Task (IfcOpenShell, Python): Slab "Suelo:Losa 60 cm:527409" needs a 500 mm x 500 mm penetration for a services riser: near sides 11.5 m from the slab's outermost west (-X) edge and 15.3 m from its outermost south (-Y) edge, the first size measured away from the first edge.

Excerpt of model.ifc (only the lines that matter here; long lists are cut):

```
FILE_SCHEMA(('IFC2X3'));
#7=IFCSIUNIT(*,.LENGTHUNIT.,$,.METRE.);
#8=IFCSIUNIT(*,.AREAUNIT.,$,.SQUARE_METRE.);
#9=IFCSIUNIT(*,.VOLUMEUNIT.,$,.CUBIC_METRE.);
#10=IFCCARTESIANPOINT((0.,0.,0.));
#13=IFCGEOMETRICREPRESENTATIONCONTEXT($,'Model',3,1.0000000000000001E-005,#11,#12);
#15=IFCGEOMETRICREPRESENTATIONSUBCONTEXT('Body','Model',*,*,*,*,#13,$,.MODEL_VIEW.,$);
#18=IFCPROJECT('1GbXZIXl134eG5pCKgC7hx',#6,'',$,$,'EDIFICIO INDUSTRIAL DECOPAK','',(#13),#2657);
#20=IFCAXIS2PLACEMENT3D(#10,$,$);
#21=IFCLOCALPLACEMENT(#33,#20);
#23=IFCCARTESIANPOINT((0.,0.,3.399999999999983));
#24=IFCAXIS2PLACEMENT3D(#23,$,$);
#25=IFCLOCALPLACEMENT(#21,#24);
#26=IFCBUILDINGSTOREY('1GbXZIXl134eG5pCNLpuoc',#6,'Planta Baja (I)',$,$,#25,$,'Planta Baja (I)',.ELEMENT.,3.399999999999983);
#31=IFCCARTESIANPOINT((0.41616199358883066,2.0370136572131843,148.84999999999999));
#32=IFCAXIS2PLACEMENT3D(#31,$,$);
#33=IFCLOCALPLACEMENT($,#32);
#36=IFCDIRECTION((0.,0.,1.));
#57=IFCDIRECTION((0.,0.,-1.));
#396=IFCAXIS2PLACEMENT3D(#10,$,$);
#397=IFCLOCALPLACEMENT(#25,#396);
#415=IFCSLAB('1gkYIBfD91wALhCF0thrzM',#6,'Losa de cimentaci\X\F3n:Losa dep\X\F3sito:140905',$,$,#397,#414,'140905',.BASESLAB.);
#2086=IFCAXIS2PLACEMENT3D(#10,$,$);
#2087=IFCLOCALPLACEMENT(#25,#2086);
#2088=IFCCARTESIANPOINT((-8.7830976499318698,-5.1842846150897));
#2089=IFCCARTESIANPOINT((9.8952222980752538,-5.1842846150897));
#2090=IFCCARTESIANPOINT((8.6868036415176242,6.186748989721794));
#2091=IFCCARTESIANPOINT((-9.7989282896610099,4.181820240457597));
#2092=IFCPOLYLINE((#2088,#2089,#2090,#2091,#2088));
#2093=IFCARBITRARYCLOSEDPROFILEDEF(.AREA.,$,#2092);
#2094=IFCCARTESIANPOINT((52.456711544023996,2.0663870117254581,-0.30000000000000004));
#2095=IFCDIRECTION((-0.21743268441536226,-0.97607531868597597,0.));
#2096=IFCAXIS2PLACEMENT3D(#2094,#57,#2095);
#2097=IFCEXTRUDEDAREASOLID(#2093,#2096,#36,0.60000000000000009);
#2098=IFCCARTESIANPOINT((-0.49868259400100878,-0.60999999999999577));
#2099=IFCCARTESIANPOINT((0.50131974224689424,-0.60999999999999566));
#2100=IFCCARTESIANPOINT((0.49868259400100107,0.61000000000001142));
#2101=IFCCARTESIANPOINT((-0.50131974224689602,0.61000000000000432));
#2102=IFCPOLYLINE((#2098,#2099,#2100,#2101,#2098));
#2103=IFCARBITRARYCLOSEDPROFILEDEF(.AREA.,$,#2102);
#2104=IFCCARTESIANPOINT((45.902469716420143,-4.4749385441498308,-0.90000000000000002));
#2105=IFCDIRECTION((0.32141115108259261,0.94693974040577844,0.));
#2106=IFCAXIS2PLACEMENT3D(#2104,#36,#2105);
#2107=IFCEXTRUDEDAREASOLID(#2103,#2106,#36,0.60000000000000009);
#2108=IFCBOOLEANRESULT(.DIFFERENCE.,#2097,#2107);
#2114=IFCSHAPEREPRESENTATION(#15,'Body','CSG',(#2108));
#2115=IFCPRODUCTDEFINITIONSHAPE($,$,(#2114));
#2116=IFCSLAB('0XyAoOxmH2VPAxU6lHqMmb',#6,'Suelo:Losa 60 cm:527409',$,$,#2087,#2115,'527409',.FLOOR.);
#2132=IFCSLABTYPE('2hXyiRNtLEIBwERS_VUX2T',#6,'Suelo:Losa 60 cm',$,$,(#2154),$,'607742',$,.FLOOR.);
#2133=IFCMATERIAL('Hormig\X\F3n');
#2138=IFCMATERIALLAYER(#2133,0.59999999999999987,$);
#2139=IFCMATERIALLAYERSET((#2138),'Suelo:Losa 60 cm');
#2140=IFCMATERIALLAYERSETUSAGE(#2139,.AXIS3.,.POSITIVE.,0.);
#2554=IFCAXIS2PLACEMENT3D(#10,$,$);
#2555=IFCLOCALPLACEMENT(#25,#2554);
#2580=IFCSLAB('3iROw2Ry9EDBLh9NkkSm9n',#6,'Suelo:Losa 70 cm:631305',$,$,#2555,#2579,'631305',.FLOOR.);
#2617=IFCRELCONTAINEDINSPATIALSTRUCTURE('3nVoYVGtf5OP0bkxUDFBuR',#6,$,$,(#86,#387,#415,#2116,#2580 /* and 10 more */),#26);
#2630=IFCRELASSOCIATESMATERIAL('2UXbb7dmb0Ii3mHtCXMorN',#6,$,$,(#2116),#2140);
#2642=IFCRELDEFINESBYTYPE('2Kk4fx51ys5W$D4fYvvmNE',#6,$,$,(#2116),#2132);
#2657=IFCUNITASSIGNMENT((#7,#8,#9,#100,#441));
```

```python
import numpy as np
import ifcopenshell
import ifcopenshell.api.feature
import ifcopenshell.api.geometry
import ifcopenshell.api.root
import ifcopenshell.geom
import ifcopenshell.util.placement
import ifcopenshell.util.representation
import ifcopenshell.util.shape
import ifcopenshell.util.unit

model = ifcopenshell.open("model.ifc")
unit_scale = ifcopenshell.util.unit.calculate_unit_scale(model)
settings = ifcopenshell.geom.settings()


def volume(element):
    """Net volume in cubic metres, openings subtracted."""
    shape = ifcopenshell.geom.create_shape(settings, element)
    return ifcopenshell.util.shape.get_volume(shape.geometry)


slab = model.by_id(2116)
before = volume(slab)

# Extent in the slab's own axes, in metres. The edges named are its -X and -Y sides.
slab_shape = ifcopenshell.geom.create_shape(settings, slab)
vertices = ifcopenshell.util.shape.get_vertices(slab_shape.geometry)
x_min, y_min, bottom = vertices.min(axis=0)
top = vertices[:, 2].max()

opening = ifcopenshell.api.root.create_entity(model, ifc_class="IfcOpeningElement", name="Services riser opening")
context = ifcopenshell.util.representation.get_context(model, "Model", "Body", "MODEL_VIEW")
width, depth = 0.5, 0.5
outline = [(0.0, 0.0), (width, 0.0), (width, depth), (0.0, depth), (0.0, 0.0)]
# Overshoot both faces by 50 mm so the cut is clean.
shape = ifcopenshell.api.geometry.add_slab_representation(
    model, context=context, depth=top - bottom + 0.1, polyline=outline
)
ifcopenshell.api.geometry.assign_representation(model, product=opening, representation=shape)

matrix = ifcopenshell.util.placement.get_local_placement(slab.ObjectPlacement)
matrix[:, 3] = matrix @ np.append(np.array([x_min + 11.5, y_min + 15.3, bottom - 0.05]) / unit_scale, 1.0)
ifcopenshell.api.geometry.edit_object_placement(model, product=opening, matrix=matrix, is_si=False)
ifcopenshell.api.feature.add_feature(model, feature=opening, element=slab)

after = volume(slab)

print(f"slab volume {before:.3f} -> {after:.3f} m3")

model.write("model_edited.ifc")
```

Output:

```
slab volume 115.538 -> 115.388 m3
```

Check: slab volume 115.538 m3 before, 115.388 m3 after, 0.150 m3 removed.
